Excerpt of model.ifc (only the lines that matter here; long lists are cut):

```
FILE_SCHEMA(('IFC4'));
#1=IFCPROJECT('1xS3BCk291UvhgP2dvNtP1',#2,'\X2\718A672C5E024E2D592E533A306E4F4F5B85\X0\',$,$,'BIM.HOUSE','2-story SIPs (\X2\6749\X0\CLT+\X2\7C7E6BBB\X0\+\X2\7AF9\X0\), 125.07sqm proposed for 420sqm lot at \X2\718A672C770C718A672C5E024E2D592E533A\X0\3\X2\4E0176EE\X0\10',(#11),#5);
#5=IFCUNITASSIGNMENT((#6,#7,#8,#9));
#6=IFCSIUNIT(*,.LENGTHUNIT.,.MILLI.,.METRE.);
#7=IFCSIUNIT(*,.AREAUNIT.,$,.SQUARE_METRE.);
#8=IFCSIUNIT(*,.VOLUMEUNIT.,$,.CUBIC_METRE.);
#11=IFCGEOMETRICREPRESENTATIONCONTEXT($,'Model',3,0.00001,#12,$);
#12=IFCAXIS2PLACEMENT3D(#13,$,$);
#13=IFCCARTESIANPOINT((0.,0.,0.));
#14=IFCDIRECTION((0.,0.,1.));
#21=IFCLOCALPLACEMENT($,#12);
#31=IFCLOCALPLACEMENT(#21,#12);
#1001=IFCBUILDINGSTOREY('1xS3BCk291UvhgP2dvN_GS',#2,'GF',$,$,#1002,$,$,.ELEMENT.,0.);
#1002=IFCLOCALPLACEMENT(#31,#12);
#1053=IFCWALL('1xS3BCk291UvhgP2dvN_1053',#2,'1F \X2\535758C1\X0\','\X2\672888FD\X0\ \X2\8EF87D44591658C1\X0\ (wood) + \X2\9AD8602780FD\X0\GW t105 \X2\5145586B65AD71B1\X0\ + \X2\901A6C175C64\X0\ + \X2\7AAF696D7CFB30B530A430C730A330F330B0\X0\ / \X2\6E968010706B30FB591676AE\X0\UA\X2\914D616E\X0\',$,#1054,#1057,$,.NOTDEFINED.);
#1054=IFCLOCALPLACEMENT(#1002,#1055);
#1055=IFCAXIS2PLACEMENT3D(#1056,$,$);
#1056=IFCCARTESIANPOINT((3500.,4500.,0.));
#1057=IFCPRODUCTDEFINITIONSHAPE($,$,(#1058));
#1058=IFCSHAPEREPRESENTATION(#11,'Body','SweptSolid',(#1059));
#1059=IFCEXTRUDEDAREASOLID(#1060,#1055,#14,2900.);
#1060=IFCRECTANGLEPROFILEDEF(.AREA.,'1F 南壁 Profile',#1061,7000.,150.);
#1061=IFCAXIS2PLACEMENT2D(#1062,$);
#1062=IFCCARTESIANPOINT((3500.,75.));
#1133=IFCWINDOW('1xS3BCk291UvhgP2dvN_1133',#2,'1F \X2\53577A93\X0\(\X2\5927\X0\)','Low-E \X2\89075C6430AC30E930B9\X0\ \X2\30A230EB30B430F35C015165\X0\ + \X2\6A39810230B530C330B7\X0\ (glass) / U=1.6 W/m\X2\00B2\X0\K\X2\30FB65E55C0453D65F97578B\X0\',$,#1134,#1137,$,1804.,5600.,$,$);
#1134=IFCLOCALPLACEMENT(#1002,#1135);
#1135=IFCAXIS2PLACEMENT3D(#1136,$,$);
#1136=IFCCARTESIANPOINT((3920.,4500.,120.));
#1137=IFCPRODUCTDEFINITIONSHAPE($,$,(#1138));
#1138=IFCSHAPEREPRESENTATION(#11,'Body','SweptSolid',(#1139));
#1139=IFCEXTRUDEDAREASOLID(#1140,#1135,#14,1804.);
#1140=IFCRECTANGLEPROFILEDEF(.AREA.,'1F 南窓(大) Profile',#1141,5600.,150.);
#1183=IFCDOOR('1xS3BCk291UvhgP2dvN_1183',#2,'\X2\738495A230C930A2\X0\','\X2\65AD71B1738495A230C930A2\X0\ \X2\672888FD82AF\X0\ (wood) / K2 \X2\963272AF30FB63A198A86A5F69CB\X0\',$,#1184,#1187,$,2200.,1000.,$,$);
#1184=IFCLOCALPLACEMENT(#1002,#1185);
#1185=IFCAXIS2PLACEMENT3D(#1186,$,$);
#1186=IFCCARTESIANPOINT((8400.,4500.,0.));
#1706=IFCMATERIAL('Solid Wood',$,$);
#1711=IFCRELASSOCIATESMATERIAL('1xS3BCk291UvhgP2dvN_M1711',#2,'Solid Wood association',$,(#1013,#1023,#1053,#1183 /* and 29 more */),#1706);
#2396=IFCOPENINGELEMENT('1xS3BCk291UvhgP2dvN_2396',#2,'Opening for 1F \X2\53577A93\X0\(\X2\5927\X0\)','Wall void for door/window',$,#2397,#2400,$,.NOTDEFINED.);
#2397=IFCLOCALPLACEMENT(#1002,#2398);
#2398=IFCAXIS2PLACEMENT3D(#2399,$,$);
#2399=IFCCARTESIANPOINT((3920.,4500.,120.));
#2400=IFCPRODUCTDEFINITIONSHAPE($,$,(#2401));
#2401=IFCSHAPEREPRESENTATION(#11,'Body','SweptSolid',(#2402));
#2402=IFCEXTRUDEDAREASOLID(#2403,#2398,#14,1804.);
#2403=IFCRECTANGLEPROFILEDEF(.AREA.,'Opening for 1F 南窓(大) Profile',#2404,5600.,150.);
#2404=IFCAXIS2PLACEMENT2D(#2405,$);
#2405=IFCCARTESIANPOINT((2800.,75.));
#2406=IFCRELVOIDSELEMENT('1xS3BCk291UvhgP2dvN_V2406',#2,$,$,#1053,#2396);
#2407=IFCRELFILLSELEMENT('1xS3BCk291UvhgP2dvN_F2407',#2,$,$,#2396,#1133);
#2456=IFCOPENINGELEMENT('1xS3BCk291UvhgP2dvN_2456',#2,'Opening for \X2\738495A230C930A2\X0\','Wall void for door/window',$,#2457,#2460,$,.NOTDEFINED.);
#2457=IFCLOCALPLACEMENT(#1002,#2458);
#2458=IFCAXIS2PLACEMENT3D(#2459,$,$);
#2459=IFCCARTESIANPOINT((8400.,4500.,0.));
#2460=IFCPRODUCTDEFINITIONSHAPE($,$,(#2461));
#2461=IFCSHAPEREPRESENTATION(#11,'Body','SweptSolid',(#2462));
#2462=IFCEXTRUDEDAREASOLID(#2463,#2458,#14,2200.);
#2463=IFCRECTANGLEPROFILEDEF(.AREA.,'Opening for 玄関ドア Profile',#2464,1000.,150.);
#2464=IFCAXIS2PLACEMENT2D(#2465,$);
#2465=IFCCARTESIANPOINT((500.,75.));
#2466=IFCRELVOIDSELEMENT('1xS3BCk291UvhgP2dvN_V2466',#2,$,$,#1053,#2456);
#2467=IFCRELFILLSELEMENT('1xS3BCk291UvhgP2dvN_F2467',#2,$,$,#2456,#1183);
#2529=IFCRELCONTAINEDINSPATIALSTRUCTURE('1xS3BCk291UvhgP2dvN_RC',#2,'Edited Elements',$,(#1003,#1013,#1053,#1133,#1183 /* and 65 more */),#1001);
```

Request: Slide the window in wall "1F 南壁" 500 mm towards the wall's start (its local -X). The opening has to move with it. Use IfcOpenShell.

```python
import ifcopenshell
import ifcopenshell.api.geometry
import ifcopenshell.util.placement

model = ifcopenshell.open("model.ifc")

window = model.by_id(1133)
opening = window.FillsVoids[0].RelatingOpeningElement
wall = opening.VoidsElements[0].RelatingBuildingElement

wall_matrix = ifcopenshell.util.placement.get_local_placement(wall.ObjectPlacement)
shift = wall_matrix[:3, 0] * -500.0
before = ifcopenshell.util.placement.get_local_placement(window.ObjectPlacement)[:3, 3].copy()

# The window is not placed relative to its opening, so move both.
for product in (opening, window):
    matrix = ifcopenshell.util.placement.get_local_placement(product.ObjectPlacement)
    matrix[:3, 3] += shift
    ifcopenshell.api.geometry.edit_object_placement(model, product=product, matrix=matrix, is_si=False)

after = ifcopenshell.util.placement.get_local_placement(window.ObjectPlacement)[:3, 3]
print("window moved by", (after - before).round(3) + 0.0)

model.write("model_v2.ifc")
```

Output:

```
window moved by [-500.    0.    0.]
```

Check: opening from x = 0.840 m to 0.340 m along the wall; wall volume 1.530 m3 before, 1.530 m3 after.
